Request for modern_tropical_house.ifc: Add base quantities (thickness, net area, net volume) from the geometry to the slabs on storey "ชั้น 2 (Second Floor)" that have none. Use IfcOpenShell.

First a look at what the model holds.

```python
import ifcopenshell
import ifcopenshell.util.element
import ifcopenshell.util.unit

model = ifcopenshell.open("modern_tropical_house.ifc")
print(model.schema)
for unit_type in ("LENGTHUNIT", "AREAUNIT", "VOLUMEUNIT"):
    print(unit_type, ifcopenshell.util.unit.calculate_unit_scale(model, unit_type))
storey = next(s for s in model.by_type("IfcBuildingStorey") if s.Name == "ชั้น 2 (Second Floor)")
slabs = [e for e in ifcopenshell.util.element.get_decomposition(storey) if e.is_a("IfcSlab")]
for e in sorted(slabs, key=lambda e: e.id()):
    print(e.id(), e.is_a(), e.Name, list(ifcopenshell.util.element.get_psets(e, qtos_only=True)), sep=" | ")
```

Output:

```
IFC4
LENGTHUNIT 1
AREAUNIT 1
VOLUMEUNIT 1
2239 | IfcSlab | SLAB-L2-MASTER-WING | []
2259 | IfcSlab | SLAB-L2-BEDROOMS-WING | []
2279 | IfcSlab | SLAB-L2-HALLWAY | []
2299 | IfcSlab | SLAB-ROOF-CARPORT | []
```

```python
import ifcopenshell
import ifcopenshell.api.pset
import ifcopenshell.geom
import ifcopenshell.util.element
import ifcopenshell.util.shape
import ifcopenshell.util.unit

model = ifcopenshell.open("modern_tropical_house.ifc")
unit_scale = ifcopenshell.util.unit.calculate_unit_scale(model)
area_scale = ifcopenshell.util.unit.calculate_unit_scale(model, "AREAUNIT")
volume_scale = ifcopenshell.util.unit.calculate_unit_scale(model, "VOLUMEUNIT")
settings = ifcopenshell.geom.settings()

storey = next(s for s in model.by_type("IfcBuildingStorey") if s.Name == "ชั้น 2 (Second Floor)")
slabs = [e for e in ifcopenshell.util.element.get_decomposition(storey) if e.is_a("IfcSlab")]

for e in sorted(slabs, key=lambda e: e.id()):
    if ifcopenshell.util.element.get_psets(e, qtos_only=True, should_inherit=False):
        continue
    # Geometry comes back in metres, in the element's own axes.
    shape = ifcopenshell.geom.create_shape(settings, e)
    values = {
        "Width": ifcopenshell.util.shape.get_z(shape.geometry) / unit_scale,
        "NetArea": ifcopenshell.util.shape.get_footprint_area(shape.geometry) / area_scale,
        "NetVolume": ifcopenshell.util.shape.get_volume(shape.geometry) / volume_scale,
    }
    qto = ifcopenshell.api.pset.add_qto(model, product=e, name="Qto_SlabBaseQuantities")
    ifcopenshell.api.pset.edit_qto(model, qto=qto, properties=values)
    print(e.id(), {k: round(v, 3) for k, v in values.items()})

model.write("modern_tropical_house_rev.ifc")
```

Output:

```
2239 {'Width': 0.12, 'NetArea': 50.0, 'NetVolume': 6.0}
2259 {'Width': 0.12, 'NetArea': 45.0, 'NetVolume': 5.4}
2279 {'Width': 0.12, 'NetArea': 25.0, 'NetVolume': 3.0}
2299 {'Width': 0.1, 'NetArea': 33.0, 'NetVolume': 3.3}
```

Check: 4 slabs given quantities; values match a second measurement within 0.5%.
